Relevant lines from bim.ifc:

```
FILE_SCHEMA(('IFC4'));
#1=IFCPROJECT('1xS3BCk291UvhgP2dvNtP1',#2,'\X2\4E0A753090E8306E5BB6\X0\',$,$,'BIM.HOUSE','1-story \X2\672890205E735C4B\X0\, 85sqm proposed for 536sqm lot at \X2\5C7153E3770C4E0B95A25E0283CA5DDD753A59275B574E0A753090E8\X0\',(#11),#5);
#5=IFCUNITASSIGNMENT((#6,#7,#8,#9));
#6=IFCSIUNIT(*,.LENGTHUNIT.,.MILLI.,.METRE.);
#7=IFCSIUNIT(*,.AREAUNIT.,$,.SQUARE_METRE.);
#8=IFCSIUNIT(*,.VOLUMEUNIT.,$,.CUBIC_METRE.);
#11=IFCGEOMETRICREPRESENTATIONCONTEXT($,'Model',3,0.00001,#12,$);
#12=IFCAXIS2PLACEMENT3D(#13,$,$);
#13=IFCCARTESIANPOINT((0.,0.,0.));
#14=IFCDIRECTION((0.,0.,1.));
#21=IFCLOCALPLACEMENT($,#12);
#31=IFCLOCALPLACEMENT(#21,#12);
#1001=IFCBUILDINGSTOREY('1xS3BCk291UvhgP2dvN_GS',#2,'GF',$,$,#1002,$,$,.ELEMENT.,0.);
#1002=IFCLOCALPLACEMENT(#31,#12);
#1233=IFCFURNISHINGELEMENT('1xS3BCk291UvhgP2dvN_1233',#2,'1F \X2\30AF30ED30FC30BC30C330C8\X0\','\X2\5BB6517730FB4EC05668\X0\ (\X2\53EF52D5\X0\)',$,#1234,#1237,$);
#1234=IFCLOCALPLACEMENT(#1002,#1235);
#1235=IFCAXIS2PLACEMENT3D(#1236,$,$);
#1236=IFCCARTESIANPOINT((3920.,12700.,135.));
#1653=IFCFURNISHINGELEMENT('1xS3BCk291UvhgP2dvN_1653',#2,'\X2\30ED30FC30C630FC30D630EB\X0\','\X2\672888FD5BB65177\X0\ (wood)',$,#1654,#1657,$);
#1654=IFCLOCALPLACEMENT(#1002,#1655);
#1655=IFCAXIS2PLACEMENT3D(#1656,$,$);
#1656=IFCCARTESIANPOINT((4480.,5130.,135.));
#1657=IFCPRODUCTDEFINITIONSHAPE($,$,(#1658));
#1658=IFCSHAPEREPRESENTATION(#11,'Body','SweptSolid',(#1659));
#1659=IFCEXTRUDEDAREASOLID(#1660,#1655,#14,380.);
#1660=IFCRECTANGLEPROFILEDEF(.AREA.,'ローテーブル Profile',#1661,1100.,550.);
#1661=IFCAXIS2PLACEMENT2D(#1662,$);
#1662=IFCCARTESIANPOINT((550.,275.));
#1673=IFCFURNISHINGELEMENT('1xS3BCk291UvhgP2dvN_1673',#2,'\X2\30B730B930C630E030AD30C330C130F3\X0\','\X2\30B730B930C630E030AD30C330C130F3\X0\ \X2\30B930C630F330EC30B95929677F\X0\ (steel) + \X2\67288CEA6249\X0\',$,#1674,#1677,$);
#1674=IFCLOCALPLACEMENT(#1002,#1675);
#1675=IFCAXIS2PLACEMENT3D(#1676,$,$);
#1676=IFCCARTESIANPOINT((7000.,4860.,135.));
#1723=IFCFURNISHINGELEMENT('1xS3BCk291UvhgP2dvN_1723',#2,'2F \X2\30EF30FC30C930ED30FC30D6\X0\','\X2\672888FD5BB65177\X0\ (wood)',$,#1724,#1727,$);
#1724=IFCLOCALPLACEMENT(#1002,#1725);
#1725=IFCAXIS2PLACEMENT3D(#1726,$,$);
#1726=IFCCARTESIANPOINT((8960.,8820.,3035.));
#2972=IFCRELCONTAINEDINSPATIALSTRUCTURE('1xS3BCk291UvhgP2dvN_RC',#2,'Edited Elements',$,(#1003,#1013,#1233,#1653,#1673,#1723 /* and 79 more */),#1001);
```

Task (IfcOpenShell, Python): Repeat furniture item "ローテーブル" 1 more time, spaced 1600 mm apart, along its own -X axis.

```python
import ifcopenshell
import ifcopenshell.api.geometry
import ifcopenshell.api.root
import ifcopenshell.util.element
import ifcopenshell.util.placement

model = ifcopenshell.open("bim.ifc")


def reuse_history(source, copy):
    """copy_class also copies each property set's owner history, people and application; keep the originals."""
    for rel in copy.IsDefinedBy:
        if rel.is_a("IfcRelDefinesByProperties") and (history := rel.RelatingPropertyDefinition.OwnerHistory):
            rel.RelatingPropertyDefinition.OwnerHistory = source.OwnerHistory
            ifcopenshell.util.element.remove_deep2(model, history)


source = model.by_guid("1xS3BCk291UvhgP2dvN_1653")
base = ifcopenshell.util.placement.get_local_placement(source.ObjectPlacement)
step = -base[:3, 0] * 1600.0

for i in range(1, 2):
    copy = ifcopenshell.api.root.copy_class(model, product=source)
    copy.Representation = ifcopenshell.util.element.copy_deep(
        model, source.Representation, exclude=["IfcGeometricRepresentationContext", "IfcRepresentationMap"]
    )
    reuse_history(source, copy)
    matrix = base.copy()
    matrix[:3, 3] += i * step
    print("added at", matrix[:3, 3].round(3) + 0.0)
    ifcopenshell.api.geometry.edit_object_placement(model, product=copy, matrix=matrix, is_si=False)

model.write("bim_edited.ifc")
```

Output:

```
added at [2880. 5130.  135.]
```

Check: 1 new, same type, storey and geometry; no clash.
